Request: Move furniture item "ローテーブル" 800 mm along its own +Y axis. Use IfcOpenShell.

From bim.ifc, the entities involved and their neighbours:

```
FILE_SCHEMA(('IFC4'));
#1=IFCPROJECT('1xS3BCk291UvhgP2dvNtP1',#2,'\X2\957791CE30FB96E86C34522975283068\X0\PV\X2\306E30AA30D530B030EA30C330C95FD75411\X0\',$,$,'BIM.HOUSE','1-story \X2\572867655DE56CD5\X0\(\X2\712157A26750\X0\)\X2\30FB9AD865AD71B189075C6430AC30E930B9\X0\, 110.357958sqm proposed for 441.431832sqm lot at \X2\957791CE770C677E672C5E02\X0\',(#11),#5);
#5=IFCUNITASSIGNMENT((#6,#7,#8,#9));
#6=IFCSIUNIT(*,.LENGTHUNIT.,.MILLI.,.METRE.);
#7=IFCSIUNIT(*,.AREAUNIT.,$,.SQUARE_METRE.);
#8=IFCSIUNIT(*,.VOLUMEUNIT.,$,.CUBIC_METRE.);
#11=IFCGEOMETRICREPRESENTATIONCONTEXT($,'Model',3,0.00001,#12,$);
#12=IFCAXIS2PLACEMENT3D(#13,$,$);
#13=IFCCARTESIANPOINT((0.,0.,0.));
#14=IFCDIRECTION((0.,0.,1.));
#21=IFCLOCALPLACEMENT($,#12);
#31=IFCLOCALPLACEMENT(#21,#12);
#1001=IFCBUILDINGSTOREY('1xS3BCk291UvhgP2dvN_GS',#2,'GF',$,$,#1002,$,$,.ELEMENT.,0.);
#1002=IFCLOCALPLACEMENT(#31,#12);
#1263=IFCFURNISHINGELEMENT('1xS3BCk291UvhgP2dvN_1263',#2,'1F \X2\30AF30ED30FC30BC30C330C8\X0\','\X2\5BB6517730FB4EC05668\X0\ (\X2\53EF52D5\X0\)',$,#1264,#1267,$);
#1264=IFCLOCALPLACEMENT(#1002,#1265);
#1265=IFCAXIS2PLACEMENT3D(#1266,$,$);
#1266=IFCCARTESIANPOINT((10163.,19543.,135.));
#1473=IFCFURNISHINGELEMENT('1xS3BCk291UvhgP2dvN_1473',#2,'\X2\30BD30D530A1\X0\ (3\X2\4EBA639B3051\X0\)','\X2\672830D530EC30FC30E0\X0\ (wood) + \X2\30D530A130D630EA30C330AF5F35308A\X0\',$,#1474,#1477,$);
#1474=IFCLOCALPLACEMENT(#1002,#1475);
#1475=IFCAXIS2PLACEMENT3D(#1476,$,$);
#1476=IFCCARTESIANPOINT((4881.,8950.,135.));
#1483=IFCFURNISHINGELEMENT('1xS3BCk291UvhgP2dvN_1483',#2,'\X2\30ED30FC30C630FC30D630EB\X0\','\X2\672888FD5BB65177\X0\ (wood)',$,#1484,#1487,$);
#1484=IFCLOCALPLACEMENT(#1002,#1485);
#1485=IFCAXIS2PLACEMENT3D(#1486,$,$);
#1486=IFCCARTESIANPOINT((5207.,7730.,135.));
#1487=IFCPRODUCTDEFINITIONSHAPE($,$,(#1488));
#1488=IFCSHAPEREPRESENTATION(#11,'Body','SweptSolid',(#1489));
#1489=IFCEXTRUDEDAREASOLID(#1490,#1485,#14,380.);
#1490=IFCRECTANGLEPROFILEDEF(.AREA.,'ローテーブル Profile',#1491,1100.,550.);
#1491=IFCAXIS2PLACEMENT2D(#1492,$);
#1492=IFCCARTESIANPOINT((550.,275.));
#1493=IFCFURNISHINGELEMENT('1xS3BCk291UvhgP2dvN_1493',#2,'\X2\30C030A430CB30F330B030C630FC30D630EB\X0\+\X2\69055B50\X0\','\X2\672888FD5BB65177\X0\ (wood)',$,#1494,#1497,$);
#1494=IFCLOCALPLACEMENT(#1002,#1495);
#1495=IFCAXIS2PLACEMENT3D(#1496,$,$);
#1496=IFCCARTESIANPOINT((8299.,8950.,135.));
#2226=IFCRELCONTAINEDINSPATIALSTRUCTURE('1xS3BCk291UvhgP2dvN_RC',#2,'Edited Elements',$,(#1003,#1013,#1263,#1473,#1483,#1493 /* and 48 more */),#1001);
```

```python
import ifcopenshell
import ifcopenshell.api.geometry
import ifcopenshell.util.placement
import ifcopenshell.util.unit

model = ifcopenshell.open("bim.ifc")
unit_scale = ifcopenshell.util.unit.calculate_unit_scale(model)

item = model.by_guid("1xS3BCk291UvhgP2dvN_1483")
matrix = ifcopenshell.util.placement.get_local_placement(item.ObjectPlacement)
matrix[:3, 3] += matrix[:3, 1] * 0.8 / unit_scale
ifcopenshell.api.geometry.edit_object_placement(model, product=item, matrix=matrix, is_si=False)

print(ifcopenshell.util.placement.get_local_placement(item.ObjectPlacement).round(3) + 0.0)

model.write("bim_rev.ifc")
```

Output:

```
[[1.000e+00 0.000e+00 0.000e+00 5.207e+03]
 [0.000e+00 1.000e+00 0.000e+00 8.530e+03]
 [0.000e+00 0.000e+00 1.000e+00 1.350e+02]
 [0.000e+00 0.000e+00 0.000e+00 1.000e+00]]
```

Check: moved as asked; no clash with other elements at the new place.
